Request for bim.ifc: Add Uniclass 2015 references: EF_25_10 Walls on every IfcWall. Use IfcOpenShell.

First a look at what the model holds.

```python
import ifcopenshell

model = ifcopenshell.open("bim.ifc")
print(model.schema)
print("classifications:", [c.Name for c in model.by_type("IfcClassification")])
for ifc_class in ("IfcDoor", "IfcRoof", "IfcStair", "IfcWall", "IfcWindow"):
    print(ifc_class, len(model.by_type(ifc_class)))
```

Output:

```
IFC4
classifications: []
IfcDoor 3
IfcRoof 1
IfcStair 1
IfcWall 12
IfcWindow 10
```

```python
import ifcopenshell
import ifcopenshell.api.classification

model = ifcopenshell.open("bim.ifc")

system = ifcopenshell.api.classification.add_classification(model, classification="Uniclass 2015")

codes = {
    "IfcWall": ("EF_25_10", "Walls"),
}
for ifc_class, (code, name) in codes.items():
    products = model.by_type(ifc_class)
    ifcopenshell.api.classification.add_reference(
        model, products=products, classification=system, identification=code, name=name
    )
    print(code, len(products))

model.write("bim_updated.ifc")
```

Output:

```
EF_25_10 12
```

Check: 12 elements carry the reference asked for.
